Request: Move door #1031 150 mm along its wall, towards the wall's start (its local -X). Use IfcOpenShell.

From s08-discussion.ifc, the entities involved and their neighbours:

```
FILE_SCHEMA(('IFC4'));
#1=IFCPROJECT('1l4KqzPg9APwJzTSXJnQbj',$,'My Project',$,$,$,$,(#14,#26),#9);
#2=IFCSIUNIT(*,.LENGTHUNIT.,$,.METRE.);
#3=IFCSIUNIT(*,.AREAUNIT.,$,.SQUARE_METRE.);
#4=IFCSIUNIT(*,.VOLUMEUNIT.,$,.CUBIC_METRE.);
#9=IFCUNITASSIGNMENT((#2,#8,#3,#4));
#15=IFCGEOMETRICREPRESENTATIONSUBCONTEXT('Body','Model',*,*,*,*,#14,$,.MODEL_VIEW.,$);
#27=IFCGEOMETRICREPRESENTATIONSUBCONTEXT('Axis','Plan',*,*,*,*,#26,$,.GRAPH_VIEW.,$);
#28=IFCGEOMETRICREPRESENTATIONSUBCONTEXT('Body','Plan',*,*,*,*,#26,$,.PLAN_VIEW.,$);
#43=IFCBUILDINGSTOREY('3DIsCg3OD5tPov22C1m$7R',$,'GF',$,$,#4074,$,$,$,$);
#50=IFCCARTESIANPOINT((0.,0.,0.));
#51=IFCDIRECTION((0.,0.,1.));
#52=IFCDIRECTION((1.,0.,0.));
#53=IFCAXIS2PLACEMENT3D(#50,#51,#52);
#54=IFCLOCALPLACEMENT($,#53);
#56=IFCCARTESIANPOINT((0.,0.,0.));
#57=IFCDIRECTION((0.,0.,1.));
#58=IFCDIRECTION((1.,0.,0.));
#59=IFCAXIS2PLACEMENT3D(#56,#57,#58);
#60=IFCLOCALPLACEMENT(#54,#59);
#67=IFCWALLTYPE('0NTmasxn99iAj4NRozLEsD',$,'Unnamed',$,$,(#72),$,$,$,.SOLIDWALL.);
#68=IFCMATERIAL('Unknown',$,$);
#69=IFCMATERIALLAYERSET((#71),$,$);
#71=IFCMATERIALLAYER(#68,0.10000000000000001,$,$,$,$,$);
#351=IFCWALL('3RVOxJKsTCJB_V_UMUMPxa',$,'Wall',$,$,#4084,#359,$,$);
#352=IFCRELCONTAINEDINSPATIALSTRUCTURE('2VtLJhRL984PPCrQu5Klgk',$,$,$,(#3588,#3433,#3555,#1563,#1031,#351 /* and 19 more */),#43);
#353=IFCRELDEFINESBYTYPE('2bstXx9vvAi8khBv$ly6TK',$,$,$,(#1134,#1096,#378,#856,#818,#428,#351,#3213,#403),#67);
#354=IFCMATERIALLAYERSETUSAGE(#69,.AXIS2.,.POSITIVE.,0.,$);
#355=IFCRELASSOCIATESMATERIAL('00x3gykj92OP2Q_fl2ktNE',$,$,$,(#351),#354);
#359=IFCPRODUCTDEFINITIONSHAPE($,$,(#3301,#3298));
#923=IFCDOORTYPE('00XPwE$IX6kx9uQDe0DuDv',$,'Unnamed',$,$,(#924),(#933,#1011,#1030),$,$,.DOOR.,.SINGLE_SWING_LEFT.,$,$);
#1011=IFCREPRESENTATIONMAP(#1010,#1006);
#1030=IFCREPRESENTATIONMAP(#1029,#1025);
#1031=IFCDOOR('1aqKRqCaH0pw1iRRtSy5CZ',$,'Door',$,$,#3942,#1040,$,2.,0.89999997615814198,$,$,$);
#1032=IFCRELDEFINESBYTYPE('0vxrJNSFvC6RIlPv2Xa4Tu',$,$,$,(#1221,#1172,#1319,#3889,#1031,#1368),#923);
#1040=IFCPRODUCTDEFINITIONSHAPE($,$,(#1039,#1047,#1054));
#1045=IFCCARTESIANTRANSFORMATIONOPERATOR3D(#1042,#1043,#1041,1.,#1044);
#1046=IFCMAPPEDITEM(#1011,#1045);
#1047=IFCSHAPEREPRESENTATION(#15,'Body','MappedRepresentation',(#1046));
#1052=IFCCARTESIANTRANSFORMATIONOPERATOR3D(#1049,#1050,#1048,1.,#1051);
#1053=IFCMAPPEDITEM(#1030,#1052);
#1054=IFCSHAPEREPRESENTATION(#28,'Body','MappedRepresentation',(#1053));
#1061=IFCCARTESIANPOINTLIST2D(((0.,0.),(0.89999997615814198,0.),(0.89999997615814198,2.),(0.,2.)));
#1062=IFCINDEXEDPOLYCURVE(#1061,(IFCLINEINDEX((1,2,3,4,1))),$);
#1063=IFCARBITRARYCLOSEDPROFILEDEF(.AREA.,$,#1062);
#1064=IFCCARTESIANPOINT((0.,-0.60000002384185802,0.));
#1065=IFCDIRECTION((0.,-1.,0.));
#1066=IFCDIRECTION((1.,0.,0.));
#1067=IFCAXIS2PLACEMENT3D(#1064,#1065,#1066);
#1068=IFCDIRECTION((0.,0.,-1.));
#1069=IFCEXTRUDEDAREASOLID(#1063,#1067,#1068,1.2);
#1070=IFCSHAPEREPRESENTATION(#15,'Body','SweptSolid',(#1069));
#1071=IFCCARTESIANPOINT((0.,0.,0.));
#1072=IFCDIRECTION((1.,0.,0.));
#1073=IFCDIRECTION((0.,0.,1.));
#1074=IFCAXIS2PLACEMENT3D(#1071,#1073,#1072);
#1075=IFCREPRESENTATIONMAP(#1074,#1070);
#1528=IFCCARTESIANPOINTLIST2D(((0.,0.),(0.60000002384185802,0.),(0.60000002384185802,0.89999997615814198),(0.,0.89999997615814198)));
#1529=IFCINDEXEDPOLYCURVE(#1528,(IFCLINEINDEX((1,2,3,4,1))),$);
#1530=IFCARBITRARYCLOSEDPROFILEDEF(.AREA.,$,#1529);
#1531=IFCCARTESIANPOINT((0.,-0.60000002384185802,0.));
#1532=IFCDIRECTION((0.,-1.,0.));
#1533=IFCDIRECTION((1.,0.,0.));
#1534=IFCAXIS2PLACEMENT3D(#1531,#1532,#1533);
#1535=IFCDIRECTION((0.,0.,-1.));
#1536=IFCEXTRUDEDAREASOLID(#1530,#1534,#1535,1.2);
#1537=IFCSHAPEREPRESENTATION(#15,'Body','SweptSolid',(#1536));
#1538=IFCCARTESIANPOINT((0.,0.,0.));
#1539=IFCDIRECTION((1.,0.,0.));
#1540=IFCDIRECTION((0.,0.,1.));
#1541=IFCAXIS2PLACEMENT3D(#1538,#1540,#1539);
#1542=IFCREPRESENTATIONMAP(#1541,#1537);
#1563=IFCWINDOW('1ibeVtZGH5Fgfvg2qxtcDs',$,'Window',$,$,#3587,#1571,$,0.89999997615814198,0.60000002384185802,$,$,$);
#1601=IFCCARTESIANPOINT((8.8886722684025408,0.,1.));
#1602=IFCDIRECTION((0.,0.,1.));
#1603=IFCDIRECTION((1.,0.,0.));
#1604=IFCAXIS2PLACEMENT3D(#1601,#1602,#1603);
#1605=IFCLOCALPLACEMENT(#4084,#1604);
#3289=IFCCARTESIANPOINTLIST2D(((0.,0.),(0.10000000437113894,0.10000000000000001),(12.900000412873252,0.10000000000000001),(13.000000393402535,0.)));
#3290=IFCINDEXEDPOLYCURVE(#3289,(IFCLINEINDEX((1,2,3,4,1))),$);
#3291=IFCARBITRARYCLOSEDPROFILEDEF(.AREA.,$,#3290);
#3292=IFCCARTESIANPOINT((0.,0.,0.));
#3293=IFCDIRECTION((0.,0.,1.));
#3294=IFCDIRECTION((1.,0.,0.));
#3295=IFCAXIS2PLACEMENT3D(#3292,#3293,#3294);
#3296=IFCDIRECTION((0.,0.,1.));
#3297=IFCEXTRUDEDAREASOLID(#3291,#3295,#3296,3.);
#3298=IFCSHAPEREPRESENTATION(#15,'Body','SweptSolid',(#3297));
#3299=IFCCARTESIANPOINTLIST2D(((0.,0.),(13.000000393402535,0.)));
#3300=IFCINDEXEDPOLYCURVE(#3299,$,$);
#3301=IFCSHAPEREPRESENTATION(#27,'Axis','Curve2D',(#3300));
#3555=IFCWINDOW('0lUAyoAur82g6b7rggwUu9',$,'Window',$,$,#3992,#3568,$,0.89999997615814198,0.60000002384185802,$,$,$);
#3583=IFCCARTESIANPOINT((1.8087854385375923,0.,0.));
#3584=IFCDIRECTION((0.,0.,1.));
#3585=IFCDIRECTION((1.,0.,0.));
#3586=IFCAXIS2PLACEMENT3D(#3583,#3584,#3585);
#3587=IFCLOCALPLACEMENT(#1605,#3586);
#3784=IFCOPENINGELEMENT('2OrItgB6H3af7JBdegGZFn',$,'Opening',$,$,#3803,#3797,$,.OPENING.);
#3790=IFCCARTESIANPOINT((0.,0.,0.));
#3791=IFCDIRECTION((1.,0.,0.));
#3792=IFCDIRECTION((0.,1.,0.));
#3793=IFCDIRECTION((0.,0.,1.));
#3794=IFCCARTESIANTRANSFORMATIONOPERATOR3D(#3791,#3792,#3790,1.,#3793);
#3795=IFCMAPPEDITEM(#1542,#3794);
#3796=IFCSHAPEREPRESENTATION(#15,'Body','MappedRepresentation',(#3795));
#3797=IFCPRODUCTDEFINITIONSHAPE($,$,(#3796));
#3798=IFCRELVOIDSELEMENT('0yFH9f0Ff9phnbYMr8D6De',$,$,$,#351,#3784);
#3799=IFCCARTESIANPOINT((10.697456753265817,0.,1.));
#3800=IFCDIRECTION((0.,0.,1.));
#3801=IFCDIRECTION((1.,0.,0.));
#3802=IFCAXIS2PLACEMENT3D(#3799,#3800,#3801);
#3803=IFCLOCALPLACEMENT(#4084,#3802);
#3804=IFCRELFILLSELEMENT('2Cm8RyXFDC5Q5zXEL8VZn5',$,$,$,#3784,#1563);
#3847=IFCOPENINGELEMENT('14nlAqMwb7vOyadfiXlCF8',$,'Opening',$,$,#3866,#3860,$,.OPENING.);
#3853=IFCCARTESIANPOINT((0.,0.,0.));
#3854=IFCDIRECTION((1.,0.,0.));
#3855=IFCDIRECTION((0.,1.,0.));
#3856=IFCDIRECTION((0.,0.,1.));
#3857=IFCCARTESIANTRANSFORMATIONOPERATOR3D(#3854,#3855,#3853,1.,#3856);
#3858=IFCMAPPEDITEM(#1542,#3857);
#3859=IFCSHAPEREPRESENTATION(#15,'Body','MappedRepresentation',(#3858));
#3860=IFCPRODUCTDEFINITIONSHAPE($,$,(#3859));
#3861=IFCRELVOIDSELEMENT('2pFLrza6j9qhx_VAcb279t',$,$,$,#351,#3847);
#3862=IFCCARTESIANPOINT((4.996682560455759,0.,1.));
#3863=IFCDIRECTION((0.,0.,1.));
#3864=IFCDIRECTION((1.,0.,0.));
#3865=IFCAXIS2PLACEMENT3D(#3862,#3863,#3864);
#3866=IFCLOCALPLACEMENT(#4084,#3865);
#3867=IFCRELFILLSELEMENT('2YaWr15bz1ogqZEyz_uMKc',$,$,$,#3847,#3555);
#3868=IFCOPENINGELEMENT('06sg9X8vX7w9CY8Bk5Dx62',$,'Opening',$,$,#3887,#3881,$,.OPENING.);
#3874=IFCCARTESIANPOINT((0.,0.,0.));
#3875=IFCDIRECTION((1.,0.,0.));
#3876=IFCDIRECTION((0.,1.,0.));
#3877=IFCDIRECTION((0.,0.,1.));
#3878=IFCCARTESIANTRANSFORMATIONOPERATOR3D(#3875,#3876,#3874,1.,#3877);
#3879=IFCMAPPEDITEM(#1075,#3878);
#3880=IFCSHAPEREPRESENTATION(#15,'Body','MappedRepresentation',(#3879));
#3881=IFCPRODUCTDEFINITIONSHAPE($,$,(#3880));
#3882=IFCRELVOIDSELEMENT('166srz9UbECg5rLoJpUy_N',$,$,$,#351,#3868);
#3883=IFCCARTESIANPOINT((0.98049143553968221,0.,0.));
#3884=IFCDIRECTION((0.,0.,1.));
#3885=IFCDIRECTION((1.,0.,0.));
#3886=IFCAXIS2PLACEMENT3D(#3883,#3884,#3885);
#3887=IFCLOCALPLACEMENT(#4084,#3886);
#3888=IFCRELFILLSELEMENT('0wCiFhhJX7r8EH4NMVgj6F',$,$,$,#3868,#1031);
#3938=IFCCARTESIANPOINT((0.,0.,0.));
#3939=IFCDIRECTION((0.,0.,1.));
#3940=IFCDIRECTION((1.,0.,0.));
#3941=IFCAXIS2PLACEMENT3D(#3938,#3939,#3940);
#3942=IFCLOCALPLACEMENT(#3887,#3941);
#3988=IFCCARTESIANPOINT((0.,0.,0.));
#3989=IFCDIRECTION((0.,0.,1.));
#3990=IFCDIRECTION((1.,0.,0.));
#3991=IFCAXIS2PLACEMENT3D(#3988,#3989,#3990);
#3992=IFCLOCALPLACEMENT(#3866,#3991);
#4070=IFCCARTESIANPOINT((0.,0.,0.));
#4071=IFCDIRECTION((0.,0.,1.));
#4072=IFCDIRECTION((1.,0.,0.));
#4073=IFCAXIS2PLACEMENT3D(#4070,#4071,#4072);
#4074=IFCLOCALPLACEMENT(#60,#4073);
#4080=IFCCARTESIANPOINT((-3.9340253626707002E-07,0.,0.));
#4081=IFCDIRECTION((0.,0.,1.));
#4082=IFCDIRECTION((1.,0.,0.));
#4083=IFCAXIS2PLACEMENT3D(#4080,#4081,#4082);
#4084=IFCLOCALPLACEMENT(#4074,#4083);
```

```python
import ifcopenshell
import ifcopenshell.api.geometry
import ifcopenshell.util.placement
import ifcopenshell.util.unit

model = ifcopenshell.open("s08-discussion.ifc")
unit_scale = ifcopenshell.util.unit.calculate_unit_scale(model)

door = model.by_guid("1aqKRqCaH0pw1iRRtSy5CZ")
opening = door.FillsVoids[0].RelatingOpeningElement
wall = opening.VoidsElements[0].RelatingBuildingElement

wall_matrix = ifcopenshell.util.placement.get_local_placement(wall.ObjectPlacement)
shift = wall_matrix[:3, 0] * -0.15 / unit_scale
before = ifcopenshell.util.placement.get_local_placement(door.ObjectPlacement)[:3, 3].copy()

# The door is placed relative to its opening, so it follows when the opening moves.
matrix = ifcopenshell.util.placement.get_local_placement(opening.ObjectPlacement)
matrix[:3, 3] += shift
ifcopenshell.api.geometry.edit_object_placement(
    model, product=opening, matrix=matrix, is_si=False, should_transform_children=True
)

after = ifcopenshell.util.placement.get_local_placement(door.ObjectPlacement)[:3, 3]
print("door moved by", (after - before).round(3) + 0.0)

model.write("s08-discussion-out.ifc")
```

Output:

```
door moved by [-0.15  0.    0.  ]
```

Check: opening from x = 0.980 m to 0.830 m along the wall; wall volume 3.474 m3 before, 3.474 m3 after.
